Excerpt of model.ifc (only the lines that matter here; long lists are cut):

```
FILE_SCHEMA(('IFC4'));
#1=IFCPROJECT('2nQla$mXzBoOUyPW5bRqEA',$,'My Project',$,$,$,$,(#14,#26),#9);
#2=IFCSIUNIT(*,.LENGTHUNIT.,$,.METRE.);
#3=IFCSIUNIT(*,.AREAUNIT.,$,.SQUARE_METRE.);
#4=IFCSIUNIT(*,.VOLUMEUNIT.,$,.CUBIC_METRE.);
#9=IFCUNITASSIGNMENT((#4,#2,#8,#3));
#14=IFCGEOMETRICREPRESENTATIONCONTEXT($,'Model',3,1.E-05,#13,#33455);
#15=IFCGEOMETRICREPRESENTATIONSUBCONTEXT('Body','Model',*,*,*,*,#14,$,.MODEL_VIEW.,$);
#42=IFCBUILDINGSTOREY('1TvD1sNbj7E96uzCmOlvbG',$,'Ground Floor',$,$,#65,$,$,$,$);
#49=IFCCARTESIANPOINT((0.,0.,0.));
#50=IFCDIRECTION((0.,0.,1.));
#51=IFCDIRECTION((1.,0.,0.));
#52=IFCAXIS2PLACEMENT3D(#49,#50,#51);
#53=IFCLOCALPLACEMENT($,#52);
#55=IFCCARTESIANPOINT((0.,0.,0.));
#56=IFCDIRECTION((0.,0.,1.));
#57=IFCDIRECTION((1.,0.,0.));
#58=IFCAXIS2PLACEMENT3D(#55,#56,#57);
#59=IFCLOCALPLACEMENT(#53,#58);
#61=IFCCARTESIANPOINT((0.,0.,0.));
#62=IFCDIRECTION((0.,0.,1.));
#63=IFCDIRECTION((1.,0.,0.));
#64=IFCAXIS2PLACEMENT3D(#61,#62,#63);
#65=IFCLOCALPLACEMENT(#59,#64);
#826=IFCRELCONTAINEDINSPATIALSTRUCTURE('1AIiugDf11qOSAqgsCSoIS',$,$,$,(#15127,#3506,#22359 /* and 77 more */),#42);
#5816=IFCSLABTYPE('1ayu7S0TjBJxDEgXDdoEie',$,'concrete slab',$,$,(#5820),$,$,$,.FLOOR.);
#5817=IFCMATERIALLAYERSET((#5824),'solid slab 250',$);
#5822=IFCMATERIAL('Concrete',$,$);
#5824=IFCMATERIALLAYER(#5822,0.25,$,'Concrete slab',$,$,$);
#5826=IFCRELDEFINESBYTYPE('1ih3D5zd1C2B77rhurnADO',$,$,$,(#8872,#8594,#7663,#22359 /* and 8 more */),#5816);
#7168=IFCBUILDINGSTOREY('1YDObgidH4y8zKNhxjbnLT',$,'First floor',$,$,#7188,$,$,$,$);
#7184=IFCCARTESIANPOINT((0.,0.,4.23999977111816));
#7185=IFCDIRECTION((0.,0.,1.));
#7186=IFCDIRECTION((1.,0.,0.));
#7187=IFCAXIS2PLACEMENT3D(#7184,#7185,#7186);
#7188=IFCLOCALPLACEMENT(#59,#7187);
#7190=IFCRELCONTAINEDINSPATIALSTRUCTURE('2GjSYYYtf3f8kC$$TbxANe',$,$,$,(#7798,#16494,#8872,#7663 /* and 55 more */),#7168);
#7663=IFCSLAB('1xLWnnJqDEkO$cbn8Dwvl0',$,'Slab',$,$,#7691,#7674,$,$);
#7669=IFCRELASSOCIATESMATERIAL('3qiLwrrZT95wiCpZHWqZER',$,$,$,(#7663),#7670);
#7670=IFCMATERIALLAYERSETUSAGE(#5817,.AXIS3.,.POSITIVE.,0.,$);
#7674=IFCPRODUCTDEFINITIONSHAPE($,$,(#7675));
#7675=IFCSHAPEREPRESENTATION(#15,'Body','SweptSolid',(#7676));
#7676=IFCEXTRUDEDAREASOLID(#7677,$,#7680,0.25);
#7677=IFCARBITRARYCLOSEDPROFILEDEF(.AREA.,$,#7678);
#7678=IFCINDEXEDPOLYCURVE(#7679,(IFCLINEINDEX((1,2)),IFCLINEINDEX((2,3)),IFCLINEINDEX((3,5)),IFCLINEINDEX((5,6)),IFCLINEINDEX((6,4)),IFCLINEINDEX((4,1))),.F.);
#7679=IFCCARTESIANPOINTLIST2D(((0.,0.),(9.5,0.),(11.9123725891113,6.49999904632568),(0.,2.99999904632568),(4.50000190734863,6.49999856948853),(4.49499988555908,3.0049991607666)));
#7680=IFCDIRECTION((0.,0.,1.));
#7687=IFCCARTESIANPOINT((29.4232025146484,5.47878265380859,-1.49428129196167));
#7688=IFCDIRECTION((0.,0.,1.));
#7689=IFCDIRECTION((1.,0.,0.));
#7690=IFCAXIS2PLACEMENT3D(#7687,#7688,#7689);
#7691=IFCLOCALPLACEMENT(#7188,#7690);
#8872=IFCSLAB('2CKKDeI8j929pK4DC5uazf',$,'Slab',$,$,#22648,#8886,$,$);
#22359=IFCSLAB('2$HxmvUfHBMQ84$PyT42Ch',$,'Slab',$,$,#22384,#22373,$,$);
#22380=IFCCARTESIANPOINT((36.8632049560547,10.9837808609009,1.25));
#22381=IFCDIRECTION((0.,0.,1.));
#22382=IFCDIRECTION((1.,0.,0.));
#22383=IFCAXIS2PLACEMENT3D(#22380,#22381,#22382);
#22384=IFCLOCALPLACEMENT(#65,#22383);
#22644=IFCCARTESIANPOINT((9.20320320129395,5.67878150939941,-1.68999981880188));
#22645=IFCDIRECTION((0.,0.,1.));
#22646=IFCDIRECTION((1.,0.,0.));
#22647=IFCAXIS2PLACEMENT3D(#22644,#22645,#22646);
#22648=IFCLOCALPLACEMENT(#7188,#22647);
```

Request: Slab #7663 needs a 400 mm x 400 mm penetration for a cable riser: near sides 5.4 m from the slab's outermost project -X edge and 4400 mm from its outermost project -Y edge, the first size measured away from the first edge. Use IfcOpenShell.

```python
import numpy as np
import ifcopenshell
import ifcopenshell.api.feature
import ifcopenshell.api.geometry
import ifcopenshell.api.root
import ifcopenshell.geom
import ifcopenshell.util.placement
import ifcopenshell.util.representation
import ifcopenshell.util.shape
import ifcopenshell.util.unit

model = ifcopenshell.open("model.ifc")
unit_scale = ifcopenshell.util.unit.calculate_unit_scale(model)
settings = ifcopenshell.geom.settings()


def volume(element):
    """Net volume in cubic metres, openings subtracted."""
    shape = ifcopenshell.geom.create_shape(settings, element)
    return ifcopenshell.util.shape.get_volume(shape.geometry)


slab = model.by_guid("1xLWnnJqDEkO$cbn8Dwvl0")
before = volume(slab)

# Extent in the slab's own axes, in metres. The edges named are its -X and -Y sides.
slab_shape = ifcopenshell.geom.create_shape(settings, slab)
vertices = ifcopenshell.util.shape.get_vertices(slab_shape.geometry)
x_min, y_min, bottom = vertices.min(axis=0)
top = vertices[:, 2].max()

opening = ifcopenshell.api.root.create_entity(model, ifc_class="IfcOpeningElement", name="Cable riser opening", predefined_type="OPENING")
context = ifcopenshell.util.representation.get_context(model, "Model", "Body", "MODEL_VIEW")
width, depth = 0.4, 0.4
outline = [(0.0, 0.0), (width, 0.0), (width, depth), (0.0, depth), (0.0, 0.0)]
# Overshoot both faces by 50 mm so the cut is clean.
shape = ifcopenshell.api.geometry.add_slab_representation(
    model, context=context, depth=top - bottom + 0.1, polyline=outline
)
ifcopenshell.api.geometry.assign_representation(model, product=opening, representation=shape)

matrix = ifcopenshell.util.placement.get_local_placement(slab.ObjectPlacement)
matrix[:, 3] = matrix @ np.append(np.array([x_min + 5.4, y_min + 4.4, bottom - 0.05]) / unit_scale, 1.0)
ifcopenshell.api.geometry.edit_object_placement(model, product=opening, matrix=matrix, is_si=False)
ifcopenshell.api.feature.add_feature(model, feature=opening, element=slab)

after = volume(slab)

print(f"slab volume {before:.3f} -> {after:.3f} m3")

model.write("model_v2.ifc")
```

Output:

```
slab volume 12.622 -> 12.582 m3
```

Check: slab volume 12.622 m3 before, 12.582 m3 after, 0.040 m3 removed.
